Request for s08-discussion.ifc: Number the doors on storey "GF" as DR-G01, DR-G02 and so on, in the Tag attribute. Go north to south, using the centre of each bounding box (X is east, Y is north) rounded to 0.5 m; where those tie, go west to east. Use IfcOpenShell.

First a look at what the model holds.

```python
import ifcopenshell
import ifcopenshell.util.element
import ifcopenshell.util.placement

model = ifcopenshell.open("s08-discussion.ifc")
print(model.schema)
storey = next(s for s in model.by_type("IfcBuildingStorey") if s.Name == "GF")
doors = [e for e in ifcopenshell.util.element.get_decomposition(storey) if e.is_a("IfcDoor")]
for e in sorted(doors, key=lambda e: e.id()):
    origin = ifcopenshell.util.placement.get_local_placement(e.ObjectPlacement)[:3, 3]
    print(e.id(), e.Tag, e.Name, origin.round(2) + 0.0, sep=" | ")
```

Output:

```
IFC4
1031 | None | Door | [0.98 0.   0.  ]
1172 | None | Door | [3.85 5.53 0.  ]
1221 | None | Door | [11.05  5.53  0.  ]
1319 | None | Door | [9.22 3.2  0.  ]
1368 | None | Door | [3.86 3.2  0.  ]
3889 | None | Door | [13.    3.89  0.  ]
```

```python
import ifcopenshell
import ifcopenshell.geom
import ifcopenshell.util.element
import ifcopenshell.util.shape

model = ifcopenshell.open("s08-discussion.ifc")
settings = ifcopenshell.geom.settings()
settings.set("use-world-coords", True)


def centre(element):
    shape = ifcopenshell.geom.create_shape(settings, element)
    return ifcopenshell.util.shape.get_bbox_centroid(shape.geometry)


storey = next(s for s in model.by_type("IfcBuildingStorey") if s.Name == "GF")
doors = [e for e in ifcopenshell.util.element.get_decomposition(storey) if e.is_a("IfcDoor")]

# Insertion points can sit at a corner or the storey origin, so sort by the geometry (in metres).
centres = {e: centre(e) for e in doors}
doors.sort(key=lambda e: (-round(centres[e][1] / 0.5), centres[e][0]))

for i, e in enumerate(doors, start=1):
    number = f"DR-G{i:02d}"
    e.Tag = number
    print(e.id(), number)

model.write("s08-discussion_rev.ifc")
```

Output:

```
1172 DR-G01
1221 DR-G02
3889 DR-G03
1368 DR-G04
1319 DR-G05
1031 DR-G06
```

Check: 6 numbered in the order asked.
